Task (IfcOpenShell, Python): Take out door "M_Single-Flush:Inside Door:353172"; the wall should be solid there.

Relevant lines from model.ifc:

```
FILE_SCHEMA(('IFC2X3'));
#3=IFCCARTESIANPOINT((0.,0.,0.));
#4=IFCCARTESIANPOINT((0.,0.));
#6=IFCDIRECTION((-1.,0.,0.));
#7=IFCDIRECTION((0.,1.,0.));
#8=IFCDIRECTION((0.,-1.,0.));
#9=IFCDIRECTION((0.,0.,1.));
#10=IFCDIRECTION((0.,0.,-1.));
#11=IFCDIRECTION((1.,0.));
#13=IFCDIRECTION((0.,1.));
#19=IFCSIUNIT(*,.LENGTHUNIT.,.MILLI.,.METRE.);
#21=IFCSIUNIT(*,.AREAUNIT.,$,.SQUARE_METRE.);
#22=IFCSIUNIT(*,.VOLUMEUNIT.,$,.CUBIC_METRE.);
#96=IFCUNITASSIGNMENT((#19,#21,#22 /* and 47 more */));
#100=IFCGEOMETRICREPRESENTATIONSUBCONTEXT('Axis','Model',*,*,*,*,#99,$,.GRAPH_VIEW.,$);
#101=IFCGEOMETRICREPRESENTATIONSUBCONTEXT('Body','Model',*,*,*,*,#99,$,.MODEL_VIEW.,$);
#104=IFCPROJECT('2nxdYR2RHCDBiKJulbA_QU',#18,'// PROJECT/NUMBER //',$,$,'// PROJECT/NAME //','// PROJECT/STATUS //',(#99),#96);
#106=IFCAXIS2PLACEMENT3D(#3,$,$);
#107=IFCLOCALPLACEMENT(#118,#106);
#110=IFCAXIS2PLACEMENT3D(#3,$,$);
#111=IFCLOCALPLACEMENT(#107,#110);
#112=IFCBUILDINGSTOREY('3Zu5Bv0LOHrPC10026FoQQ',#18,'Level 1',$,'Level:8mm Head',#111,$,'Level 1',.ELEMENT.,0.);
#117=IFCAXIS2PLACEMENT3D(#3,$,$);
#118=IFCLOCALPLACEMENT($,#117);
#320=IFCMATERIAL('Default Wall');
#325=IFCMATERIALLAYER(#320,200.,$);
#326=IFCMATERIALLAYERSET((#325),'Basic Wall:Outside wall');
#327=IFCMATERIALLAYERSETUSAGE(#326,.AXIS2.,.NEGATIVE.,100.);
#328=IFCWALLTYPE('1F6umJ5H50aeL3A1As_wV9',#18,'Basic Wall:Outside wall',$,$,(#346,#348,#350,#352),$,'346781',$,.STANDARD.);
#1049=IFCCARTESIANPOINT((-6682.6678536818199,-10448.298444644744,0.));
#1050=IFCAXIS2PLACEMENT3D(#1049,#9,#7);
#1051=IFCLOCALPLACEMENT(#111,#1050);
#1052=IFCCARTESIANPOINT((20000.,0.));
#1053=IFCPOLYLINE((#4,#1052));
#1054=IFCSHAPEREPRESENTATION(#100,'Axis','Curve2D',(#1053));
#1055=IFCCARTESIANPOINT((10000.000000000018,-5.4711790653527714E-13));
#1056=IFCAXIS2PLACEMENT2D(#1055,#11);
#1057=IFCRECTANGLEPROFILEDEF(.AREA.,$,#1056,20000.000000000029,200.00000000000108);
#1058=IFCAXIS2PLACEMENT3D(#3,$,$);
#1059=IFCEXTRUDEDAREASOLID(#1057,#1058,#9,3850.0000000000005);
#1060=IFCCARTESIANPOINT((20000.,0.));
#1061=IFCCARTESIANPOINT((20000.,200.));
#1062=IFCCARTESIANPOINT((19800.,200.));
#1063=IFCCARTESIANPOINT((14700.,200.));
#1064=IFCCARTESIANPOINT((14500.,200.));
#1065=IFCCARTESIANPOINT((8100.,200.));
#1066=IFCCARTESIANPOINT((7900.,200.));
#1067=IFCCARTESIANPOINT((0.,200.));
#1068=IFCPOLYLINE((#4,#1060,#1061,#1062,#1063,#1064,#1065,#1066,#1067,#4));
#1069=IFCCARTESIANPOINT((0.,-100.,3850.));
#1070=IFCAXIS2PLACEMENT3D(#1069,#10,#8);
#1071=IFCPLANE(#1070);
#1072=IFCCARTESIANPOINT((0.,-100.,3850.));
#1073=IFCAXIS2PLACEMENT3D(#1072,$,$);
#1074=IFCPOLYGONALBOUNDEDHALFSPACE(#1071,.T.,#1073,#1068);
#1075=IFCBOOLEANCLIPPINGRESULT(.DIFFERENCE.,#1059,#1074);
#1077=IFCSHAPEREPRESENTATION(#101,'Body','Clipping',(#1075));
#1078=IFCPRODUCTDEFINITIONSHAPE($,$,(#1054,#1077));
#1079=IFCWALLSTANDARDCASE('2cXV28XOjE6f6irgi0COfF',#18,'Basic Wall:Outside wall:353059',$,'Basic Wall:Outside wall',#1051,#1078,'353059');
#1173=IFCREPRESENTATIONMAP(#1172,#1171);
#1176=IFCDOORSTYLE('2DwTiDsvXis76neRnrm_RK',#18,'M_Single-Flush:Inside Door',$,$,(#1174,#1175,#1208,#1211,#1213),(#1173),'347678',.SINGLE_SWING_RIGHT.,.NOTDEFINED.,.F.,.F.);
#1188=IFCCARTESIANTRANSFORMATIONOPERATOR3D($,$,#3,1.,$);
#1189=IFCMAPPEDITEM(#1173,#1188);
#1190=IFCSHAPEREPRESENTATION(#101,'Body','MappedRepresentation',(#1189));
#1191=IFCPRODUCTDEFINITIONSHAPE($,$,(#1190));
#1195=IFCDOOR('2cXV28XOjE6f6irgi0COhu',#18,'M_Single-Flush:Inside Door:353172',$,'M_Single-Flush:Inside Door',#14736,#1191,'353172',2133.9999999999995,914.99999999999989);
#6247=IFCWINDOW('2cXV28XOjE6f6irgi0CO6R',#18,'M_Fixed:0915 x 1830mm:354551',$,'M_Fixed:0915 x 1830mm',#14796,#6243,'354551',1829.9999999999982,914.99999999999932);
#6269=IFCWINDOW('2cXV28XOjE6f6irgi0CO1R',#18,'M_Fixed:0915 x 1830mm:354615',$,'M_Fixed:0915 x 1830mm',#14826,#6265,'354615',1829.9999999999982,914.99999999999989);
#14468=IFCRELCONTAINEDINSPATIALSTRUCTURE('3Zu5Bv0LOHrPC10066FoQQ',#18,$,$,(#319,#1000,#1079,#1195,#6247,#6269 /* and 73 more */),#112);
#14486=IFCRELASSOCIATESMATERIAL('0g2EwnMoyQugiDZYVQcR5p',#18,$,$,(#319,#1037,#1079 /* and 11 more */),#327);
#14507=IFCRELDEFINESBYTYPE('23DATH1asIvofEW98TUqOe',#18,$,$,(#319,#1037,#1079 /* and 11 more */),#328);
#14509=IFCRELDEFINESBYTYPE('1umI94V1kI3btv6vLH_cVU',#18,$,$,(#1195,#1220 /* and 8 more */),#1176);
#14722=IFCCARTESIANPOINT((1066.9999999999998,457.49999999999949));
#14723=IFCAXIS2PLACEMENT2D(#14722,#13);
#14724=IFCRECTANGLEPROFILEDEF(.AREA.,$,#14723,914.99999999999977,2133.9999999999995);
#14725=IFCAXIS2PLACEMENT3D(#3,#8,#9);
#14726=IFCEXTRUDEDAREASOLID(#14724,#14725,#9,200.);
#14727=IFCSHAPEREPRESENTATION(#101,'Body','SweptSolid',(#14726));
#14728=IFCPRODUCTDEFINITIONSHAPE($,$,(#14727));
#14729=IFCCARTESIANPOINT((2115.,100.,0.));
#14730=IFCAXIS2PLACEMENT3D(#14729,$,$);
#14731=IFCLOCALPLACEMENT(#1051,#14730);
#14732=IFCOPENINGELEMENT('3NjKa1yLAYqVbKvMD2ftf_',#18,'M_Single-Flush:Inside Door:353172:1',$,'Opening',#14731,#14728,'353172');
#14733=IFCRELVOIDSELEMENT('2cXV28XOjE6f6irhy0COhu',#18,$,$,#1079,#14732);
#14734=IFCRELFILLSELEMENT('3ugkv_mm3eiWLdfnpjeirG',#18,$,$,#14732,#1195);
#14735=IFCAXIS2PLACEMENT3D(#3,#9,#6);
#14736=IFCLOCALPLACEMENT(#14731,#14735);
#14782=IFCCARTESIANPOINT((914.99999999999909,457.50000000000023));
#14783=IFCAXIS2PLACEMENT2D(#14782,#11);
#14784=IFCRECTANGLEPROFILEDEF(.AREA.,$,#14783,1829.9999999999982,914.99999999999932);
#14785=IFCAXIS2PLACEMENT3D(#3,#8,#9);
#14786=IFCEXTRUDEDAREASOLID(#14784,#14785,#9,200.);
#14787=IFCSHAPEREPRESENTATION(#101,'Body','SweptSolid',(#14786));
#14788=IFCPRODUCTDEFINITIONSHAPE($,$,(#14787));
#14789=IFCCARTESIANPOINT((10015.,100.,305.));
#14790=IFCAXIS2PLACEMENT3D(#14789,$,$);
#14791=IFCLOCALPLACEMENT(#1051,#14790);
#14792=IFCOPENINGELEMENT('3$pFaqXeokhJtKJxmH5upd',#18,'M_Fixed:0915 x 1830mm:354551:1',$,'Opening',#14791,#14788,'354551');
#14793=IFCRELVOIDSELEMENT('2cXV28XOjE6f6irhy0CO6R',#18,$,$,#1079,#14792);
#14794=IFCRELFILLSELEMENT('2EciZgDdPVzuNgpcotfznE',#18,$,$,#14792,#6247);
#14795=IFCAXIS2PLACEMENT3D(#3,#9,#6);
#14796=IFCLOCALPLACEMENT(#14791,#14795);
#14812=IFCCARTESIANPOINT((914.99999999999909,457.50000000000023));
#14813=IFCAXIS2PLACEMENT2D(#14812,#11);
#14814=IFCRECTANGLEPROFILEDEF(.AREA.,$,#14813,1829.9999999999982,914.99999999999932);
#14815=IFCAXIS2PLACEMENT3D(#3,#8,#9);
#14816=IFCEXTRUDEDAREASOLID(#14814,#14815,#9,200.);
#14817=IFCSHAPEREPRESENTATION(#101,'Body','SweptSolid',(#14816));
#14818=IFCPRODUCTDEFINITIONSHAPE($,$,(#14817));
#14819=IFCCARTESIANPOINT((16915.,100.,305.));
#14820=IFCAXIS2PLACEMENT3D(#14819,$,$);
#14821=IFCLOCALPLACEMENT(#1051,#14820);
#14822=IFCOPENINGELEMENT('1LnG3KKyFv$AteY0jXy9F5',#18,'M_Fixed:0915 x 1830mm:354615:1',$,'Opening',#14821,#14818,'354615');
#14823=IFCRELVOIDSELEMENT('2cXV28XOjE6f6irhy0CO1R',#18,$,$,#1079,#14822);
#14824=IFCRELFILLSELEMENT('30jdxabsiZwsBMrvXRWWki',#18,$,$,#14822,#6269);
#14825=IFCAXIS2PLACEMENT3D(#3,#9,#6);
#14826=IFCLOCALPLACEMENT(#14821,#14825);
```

```python
import ifcopenshell
import ifcopenshell.api.feature
import ifcopenshell.api.root
import ifcopenshell.geom
import ifcopenshell.util.shape

model = ifcopenshell.open("model.ifc")
settings = ifcopenshell.geom.settings()


def volume(element):
    """Net volume in cubic metres, openings subtracted."""
    shape = ifcopenshell.geom.create_shape(settings, element)
    return ifcopenshell.util.shape.get_volume(shape.geometry)


door = model.by_id(1195)
opening = door.FillsVoids[0].RelatingOpeningElement
wall = opening.VoidsElements[0].RelatingBuildingElement
before = volume(wall)

ifcopenshell.api.root.remove_product(model, product=door)
ifcopenshell.api.feature.remove_feature(model, feature=opening)

after = volume(wall)

print(f"wall volume {before:.3f} -> {after:.3f} m3")

model.write("model_rev.ifc")
```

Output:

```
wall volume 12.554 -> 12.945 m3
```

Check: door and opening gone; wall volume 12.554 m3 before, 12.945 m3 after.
